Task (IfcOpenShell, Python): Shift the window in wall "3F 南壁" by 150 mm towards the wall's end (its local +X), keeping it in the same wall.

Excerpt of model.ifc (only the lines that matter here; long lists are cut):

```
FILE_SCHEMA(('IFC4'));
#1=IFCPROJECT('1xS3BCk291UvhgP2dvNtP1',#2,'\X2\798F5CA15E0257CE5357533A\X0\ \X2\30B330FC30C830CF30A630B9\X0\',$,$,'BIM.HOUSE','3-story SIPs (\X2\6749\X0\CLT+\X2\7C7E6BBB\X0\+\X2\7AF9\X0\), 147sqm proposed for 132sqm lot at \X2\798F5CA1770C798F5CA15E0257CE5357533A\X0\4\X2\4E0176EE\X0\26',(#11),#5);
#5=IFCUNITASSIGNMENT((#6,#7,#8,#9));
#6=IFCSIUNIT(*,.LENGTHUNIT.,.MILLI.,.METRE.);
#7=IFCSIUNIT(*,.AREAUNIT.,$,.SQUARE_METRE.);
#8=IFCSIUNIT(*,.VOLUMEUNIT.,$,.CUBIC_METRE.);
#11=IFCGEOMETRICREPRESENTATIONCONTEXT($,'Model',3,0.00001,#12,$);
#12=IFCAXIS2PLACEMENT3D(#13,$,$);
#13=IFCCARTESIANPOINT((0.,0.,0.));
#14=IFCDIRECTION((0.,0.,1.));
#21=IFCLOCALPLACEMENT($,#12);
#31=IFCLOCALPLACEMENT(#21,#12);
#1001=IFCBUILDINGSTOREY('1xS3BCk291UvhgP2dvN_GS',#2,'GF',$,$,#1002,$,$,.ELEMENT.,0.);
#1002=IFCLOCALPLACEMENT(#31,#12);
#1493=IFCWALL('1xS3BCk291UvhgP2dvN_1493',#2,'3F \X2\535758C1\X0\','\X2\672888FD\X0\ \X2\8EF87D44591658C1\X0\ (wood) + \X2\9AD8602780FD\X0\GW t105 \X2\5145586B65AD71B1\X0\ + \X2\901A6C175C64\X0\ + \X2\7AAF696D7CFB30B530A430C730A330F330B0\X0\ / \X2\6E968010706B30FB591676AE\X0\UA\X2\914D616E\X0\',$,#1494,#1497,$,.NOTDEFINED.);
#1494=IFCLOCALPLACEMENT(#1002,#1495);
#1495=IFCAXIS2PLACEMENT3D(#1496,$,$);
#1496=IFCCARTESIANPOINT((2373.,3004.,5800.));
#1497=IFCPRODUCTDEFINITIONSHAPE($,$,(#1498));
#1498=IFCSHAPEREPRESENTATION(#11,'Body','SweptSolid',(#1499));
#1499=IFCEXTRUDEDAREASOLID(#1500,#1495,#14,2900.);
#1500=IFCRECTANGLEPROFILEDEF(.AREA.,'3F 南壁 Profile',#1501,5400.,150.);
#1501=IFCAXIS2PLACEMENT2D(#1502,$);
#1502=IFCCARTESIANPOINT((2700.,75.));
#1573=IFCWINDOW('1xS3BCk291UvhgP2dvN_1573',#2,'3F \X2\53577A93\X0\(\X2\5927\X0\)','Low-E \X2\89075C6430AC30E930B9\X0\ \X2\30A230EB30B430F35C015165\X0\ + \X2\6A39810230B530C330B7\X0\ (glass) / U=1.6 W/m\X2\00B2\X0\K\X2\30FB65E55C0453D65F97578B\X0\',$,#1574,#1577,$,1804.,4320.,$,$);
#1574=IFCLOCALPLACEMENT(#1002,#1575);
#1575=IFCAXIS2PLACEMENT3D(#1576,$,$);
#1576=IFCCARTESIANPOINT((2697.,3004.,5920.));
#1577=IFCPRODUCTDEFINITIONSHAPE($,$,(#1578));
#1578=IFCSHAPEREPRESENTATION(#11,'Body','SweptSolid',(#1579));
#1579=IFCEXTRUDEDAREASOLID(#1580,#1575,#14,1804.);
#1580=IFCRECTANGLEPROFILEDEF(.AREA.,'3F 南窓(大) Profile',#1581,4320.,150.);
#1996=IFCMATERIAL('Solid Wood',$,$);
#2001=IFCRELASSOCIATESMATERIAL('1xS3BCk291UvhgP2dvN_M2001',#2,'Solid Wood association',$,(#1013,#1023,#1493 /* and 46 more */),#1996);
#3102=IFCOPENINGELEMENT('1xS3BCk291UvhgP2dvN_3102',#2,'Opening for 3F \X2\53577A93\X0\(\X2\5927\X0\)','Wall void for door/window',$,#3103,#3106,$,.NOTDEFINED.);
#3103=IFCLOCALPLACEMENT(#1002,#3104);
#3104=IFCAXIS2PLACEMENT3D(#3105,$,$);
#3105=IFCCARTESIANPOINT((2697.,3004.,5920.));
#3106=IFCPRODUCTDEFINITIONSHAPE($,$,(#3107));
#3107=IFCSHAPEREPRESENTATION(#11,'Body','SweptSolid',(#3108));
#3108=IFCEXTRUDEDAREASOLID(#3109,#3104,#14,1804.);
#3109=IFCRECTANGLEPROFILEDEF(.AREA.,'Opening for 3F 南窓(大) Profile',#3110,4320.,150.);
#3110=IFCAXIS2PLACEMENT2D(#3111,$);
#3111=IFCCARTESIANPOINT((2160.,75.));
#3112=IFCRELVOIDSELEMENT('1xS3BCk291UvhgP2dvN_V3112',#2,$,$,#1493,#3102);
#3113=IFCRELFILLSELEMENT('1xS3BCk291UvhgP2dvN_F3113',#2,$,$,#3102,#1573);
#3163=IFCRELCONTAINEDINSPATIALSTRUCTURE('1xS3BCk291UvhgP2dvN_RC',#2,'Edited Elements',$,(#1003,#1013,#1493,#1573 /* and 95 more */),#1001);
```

```python
import ifcopenshell
import ifcopenshell.api.geometry
import ifcopenshell.util.placement

model = ifcopenshell.open("model.ifc")

window = model.by_guid("1xS3BCk291UvhgP2dvN_1573")
opening = window.FillsVoids[0].RelatingOpeningElement
wall = opening.VoidsElements[0].RelatingBuildingElement

wall_matrix = ifcopenshell.util.placement.get_local_placement(wall.ObjectPlacement)
shift = wall_matrix[:3, 0] * 150.0
before = ifcopenshell.util.placement.get_local_placement(window.ObjectPlacement)[:3, 3].copy()

# The window is not placed relative to its opening, so move both.
for product in (opening, window):
    matrix = ifcopenshell.util.placement.get_local_placement(product.ObjectPlacement)
    matrix[:3, 3] += shift
    ifcopenshell.api.geometry.edit_object_placement(model, product=product, matrix=matrix, is_si=False)

after = ifcopenshell.util.placement.get_local_placement(window.ObjectPlacement)[:3, 3]
print("window moved by", (after - before).round(3) + 0.0)

model.write("model_v2.ifc")
```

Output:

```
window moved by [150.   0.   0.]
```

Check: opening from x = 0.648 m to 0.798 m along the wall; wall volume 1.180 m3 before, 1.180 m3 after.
